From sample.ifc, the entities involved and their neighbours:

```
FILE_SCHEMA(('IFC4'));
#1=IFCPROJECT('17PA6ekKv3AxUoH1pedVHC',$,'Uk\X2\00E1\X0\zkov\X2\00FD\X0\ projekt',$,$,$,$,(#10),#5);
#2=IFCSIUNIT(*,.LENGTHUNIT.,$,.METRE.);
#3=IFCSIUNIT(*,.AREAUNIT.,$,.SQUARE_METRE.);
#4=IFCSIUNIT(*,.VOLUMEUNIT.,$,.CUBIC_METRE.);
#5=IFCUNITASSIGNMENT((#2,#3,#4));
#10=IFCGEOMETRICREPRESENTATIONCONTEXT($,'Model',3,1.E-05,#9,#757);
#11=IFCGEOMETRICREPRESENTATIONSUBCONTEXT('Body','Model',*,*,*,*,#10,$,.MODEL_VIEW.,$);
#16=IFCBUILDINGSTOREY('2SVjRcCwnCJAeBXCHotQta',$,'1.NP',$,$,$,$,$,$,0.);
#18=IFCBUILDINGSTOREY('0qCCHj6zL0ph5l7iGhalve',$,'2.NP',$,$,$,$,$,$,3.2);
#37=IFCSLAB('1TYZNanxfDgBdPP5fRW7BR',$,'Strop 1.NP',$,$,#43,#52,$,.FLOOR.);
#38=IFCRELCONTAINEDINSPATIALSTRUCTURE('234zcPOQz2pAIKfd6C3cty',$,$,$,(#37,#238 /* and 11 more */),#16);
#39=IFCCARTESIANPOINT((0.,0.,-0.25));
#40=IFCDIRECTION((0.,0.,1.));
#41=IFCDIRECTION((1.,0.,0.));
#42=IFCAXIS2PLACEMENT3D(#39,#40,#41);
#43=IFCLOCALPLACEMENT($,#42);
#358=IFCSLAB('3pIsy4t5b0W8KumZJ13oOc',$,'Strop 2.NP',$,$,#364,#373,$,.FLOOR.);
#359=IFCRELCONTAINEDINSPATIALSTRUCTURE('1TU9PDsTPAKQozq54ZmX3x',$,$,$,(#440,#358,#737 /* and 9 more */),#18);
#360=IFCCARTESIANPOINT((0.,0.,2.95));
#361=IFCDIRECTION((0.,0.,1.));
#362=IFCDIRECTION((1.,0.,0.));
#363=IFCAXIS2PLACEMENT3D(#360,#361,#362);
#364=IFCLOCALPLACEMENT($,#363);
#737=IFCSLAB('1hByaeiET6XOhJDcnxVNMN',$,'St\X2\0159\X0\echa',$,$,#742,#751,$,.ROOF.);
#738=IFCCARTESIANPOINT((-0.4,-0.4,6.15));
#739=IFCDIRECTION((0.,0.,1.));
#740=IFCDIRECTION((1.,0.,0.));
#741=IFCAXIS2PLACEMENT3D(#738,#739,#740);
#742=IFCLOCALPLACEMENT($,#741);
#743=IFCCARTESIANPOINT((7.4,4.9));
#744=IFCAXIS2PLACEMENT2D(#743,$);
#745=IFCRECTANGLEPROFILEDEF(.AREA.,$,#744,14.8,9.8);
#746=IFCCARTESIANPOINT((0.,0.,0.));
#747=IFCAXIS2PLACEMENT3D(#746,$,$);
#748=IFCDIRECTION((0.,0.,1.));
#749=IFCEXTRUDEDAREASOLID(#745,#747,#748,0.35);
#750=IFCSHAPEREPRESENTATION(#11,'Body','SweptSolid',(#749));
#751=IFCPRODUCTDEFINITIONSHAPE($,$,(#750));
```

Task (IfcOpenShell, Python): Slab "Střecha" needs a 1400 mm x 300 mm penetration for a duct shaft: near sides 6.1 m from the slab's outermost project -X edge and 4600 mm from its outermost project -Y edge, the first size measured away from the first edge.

```python
import numpy as np
import ifcopenshell
import ifcopenshell.api.feature
import ifcopenshell.api.geometry
import ifcopenshell.api.root
import ifcopenshell.geom
import ifcopenshell.util.placement
import ifcopenshell.util.representation
import ifcopenshell.util.shape
import ifcopenshell.util.unit

model = ifcopenshell.open("sample.ifc")
unit_scale = ifcopenshell.util.unit.calculate_unit_scale(model)
settings = ifcopenshell.geom.settings()


def volume(element):
    """Net volume in cubic metres, openings subtracted."""
    shape = ifcopenshell.geom.create_shape(settings, element)
    return ifcopenshell.util.shape.get_volume(shape.geometry)


slab = model.by_guid("1hByaeiET6XOhJDcnxVNMN")
before = volume(slab)

# Extent in the slab's own axes, in metres. The edges named are its -X and -Y sides.
slab_shape = ifcopenshell.geom.create_shape(settings, slab)
vertices = ifcopenshell.util.shape.get_vertices(slab_shape.geometry)
x_min, y_min, bottom = vertices.min(axis=0)
top = vertices[:, 2].max()

opening = ifcopenshell.api.root.create_entity(model, ifc_class="IfcOpeningElement", name="Duct shaft opening", predefined_type="OPENING")
context = ifcopenshell.util.representation.get_context(model, "Model", "Body", "MODEL_VIEW")
width, depth = 1.4, 0.3
outline = [(0.0, 0.0), (width, 0.0), (width, depth), (0.0, depth), (0.0, 0.0)]
# Overshoot both faces by 50 mm so the cut is clean.
shape = ifcopenshell.api.geometry.add_slab_representation(
    model, context=context, depth=top - bottom + 0.1, polyline=outline
)
ifcopenshell.api.geometry.assign_representation(model, product=opening, representation=shape)

matrix = ifcopenshell.util.placement.get_local_placement(slab.ObjectPlacement)
matrix[:, 3] = matrix @ np.append(np.array([x_min + 6.1, y_min + 4.6, bottom - 0.05]) / unit_scale, 1.0)
ifcopenshell.api.geometry.edit_object_placement(model, product=opening, matrix=matrix, is_si=False)
ifcopenshell.api.feature.add_feature(model, feature=opening, element=slab)

after = volume(slab)

print(f"slab volume {before:.3f} -> {after:.3f} m3")

model.write("sample_v2.ifc")
```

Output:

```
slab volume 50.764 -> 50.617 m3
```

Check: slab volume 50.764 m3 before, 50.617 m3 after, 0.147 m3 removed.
